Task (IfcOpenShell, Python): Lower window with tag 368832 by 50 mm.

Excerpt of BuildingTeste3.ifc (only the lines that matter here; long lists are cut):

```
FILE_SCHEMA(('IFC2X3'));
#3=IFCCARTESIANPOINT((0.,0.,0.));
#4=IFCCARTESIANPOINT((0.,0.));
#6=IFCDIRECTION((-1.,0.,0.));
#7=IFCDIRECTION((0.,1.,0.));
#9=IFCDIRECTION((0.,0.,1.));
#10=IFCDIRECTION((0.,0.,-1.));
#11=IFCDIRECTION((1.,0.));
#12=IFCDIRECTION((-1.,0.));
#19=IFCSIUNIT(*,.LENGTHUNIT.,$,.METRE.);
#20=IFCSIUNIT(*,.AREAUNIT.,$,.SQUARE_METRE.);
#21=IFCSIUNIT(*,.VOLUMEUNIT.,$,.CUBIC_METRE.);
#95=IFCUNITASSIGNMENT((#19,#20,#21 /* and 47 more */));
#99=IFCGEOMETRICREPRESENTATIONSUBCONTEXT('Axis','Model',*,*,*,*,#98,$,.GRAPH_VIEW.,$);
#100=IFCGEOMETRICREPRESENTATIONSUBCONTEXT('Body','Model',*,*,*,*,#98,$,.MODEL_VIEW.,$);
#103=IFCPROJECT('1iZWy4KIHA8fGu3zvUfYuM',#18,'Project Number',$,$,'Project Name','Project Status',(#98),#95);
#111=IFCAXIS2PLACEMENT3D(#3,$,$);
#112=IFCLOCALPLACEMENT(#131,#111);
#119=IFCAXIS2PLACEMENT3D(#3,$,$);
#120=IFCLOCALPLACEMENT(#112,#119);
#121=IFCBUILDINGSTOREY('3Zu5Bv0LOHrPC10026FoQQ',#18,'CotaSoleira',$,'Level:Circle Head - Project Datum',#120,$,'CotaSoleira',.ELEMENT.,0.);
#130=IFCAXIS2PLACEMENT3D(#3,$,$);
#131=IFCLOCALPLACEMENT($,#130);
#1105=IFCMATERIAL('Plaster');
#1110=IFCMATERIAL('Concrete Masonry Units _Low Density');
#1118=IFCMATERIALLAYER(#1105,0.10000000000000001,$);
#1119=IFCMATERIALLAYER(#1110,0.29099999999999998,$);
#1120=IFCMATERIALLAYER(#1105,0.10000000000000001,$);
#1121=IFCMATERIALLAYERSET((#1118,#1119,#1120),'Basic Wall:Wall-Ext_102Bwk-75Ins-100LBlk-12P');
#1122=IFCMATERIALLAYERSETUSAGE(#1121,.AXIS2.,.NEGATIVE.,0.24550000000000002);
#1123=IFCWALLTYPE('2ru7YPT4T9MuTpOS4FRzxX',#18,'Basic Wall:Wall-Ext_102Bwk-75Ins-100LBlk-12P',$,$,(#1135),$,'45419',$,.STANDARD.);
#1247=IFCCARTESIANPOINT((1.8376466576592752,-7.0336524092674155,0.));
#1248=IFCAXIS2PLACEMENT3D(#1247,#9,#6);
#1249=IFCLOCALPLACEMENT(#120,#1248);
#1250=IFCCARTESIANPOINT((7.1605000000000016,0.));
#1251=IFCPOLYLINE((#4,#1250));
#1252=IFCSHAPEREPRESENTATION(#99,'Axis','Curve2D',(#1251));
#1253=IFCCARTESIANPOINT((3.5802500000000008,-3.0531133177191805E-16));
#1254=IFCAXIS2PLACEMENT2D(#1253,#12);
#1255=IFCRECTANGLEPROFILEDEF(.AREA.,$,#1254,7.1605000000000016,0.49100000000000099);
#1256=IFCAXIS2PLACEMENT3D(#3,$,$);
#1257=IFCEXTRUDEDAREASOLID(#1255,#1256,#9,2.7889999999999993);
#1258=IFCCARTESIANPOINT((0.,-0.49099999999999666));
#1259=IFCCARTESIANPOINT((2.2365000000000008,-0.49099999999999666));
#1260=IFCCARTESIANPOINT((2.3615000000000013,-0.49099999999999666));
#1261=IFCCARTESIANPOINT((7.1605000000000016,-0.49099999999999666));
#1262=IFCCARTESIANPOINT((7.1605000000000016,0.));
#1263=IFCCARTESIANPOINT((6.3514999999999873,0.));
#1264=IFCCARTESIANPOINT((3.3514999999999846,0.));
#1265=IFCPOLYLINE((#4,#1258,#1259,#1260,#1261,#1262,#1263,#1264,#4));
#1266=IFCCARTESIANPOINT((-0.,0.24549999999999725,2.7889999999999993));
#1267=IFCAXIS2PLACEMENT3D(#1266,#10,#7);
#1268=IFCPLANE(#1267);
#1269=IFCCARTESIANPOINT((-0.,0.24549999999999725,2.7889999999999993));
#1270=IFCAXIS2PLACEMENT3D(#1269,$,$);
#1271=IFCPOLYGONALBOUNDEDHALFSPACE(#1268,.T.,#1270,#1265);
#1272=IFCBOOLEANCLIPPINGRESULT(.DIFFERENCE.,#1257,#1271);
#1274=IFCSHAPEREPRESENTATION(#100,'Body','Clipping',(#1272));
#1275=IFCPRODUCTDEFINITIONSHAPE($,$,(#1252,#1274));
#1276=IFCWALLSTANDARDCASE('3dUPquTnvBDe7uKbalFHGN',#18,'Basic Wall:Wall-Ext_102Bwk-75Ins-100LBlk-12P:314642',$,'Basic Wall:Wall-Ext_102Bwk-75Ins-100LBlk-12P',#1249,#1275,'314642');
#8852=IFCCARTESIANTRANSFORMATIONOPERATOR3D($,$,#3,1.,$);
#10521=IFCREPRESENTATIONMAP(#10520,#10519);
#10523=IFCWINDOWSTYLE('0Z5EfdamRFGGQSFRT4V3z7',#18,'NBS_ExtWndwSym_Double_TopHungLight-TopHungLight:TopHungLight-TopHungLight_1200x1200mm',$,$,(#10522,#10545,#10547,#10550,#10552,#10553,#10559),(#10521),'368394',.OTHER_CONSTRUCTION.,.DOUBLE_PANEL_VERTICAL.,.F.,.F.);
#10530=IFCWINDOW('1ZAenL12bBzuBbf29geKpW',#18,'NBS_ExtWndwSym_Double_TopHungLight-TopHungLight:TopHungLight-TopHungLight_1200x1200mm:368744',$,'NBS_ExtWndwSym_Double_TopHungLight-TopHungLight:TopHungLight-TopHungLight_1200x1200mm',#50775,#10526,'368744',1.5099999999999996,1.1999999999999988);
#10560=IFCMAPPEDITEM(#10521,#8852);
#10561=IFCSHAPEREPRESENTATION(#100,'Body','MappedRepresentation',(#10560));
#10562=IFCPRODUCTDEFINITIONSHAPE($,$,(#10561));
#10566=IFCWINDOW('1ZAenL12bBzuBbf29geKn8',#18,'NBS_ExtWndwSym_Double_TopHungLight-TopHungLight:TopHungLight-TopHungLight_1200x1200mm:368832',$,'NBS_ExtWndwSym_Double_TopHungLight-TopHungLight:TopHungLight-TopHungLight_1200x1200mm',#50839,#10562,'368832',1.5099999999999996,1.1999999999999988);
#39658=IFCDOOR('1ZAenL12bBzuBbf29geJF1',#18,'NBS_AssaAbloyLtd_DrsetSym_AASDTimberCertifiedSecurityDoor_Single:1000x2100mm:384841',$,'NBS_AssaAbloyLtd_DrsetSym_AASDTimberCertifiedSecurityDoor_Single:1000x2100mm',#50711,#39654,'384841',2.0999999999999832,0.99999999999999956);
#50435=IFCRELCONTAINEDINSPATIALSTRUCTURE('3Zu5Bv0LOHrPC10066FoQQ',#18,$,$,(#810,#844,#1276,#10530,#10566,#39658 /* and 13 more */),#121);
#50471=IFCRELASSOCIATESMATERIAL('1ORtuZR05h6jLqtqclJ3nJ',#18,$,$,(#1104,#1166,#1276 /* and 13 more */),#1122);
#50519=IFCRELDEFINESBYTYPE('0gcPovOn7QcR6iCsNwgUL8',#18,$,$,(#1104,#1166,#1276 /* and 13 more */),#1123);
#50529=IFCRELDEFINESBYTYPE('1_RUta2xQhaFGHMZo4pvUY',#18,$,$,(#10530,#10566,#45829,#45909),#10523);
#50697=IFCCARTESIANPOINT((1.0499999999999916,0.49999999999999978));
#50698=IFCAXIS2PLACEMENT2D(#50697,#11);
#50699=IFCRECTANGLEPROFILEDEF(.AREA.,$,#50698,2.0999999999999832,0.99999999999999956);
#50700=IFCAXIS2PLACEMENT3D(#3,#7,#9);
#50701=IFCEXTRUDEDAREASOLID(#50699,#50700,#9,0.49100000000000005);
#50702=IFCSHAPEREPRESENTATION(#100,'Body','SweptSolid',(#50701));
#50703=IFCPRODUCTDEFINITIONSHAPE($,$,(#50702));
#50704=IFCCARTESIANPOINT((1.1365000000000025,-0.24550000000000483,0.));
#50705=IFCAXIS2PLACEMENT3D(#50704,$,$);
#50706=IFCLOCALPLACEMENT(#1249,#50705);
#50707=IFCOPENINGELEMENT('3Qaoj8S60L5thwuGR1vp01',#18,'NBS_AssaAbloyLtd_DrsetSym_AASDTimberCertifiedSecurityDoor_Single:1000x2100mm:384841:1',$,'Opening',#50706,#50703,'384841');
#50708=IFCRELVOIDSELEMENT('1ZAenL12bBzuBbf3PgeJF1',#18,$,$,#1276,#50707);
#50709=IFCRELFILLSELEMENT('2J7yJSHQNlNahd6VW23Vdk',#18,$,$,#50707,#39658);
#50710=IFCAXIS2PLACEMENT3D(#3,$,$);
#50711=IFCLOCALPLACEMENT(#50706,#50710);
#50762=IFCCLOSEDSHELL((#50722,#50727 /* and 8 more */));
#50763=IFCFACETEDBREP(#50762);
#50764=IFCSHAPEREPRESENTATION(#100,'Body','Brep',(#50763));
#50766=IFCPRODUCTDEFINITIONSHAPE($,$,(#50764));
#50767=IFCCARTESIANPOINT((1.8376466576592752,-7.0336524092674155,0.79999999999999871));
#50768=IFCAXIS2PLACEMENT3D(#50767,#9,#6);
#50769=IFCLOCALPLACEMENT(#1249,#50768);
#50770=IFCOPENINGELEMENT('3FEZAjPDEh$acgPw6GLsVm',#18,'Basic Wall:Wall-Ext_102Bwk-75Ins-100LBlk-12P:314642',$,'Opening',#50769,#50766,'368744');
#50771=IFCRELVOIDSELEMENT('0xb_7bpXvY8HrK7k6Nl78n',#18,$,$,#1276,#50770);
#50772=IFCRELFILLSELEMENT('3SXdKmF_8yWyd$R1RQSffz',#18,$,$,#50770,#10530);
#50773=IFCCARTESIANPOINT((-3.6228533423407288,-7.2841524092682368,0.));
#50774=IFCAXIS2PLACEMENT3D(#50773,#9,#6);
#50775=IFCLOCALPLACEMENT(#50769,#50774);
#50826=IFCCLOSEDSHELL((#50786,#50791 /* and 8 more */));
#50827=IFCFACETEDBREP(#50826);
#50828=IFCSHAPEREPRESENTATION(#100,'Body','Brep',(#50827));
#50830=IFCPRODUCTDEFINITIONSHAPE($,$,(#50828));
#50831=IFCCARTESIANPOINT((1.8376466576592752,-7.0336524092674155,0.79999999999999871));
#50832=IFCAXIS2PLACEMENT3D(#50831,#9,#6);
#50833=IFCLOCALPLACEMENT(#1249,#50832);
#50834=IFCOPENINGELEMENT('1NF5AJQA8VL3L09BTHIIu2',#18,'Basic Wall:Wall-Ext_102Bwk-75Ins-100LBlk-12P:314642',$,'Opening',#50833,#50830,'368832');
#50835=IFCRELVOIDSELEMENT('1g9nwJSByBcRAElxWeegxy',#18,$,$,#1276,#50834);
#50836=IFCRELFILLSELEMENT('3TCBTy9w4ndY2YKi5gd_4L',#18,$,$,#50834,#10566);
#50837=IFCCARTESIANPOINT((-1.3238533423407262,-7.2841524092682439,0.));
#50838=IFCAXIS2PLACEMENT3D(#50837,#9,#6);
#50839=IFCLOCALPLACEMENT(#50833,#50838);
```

```python
import numpy as np
import ifcopenshell
import ifcopenshell.api.geometry
import ifcopenshell.util.placement
import ifcopenshell.util.unit

model = ifcopenshell.open("BuildingTeste3.ifc")
unit_scale = ifcopenshell.util.unit.calculate_unit_scale(model)

window = model.by_guid("1ZAenL12bBzuBbf29geKn8")
opening = window.FillsVoids[0].RelatingOpeningElement
dz = -0.05

shift = np.array([0.0, 0.0, dz])
# The window is placed relative to its opening, so it follows when the opening moves.
matrix = ifcopenshell.util.placement.get_local_placement(opening.ObjectPlacement)
matrix[:3, 3] += shift
ifcopenshell.api.geometry.edit_object_placement(
    model, product=opening, matrix=matrix, is_si=False, should_transform_children=True
)

print(f"moved by {dz * unit_scale:+.3f} m")

model.write("BuildingTeste3_v2.ifc")
```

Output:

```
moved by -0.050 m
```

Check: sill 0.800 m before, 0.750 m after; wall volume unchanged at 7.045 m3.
